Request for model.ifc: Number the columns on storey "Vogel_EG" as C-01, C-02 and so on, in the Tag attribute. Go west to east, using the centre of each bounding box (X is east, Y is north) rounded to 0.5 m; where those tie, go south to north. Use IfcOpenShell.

First a look at what the model holds.

```python
import ifcopenshell
import ifcopenshell.util.element
import ifcopenshell.util.placement

model = ifcopenshell.open("model.ifc")
print(model.schema)
storey = next(s for s in model.by_type("IfcBuildingStorey") if s.Name == "Vogel_EG")
columns = [e for e in ifcopenshell.util.element.get_decomposition(storey) if e.is_a("IfcColumn")]
for e in sorted(columns, key=lambda e: e.id()):
    origin = ifcopenshell.util.placement.get_local_placement(e.ObjectPlacement)[:3, 3]
    print(e.id(), e.Tag, e.Name, origin.round(2) + 0.0, sep=" | ")
```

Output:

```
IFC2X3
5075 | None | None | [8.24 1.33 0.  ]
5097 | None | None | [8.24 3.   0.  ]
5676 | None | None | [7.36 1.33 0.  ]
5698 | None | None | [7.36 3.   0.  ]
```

```python
import ifcopenshell
import ifcopenshell.geom
import ifcopenshell.util.element
import ifcopenshell.util.shape

model = ifcopenshell.open("model.ifc")
settings = ifcopenshell.geom.settings()
settings.set("use-world-coords", True)


def centre(element):
    shape = ifcopenshell.geom.create_shape(settings, element)
    return ifcopenshell.util.shape.get_bbox_centroid(shape.geometry)


storey = next(s for s in model.by_type("IfcBuildingStorey") if s.Name == "Vogel_EG")
columns = [e for e in ifcopenshell.util.element.get_decomposition(storey) if e.is_a("IfcColumn")]

# Insertion points can sit at a corner or the storey origin, so sort by the geometry (in metres).
centres = {e: centre(e) for e in columns}
columns.sort(key=lambda e: (round(centres[e][0] / 0.5), centres[e][1]))

for i, e in enumerate(columns, start=1):
    number = f"C-{i:02d}"
    e.Tag = number
    print(e.id(), number)

model.write("model_rev.ifc")
```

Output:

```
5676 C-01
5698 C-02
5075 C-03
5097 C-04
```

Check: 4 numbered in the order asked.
